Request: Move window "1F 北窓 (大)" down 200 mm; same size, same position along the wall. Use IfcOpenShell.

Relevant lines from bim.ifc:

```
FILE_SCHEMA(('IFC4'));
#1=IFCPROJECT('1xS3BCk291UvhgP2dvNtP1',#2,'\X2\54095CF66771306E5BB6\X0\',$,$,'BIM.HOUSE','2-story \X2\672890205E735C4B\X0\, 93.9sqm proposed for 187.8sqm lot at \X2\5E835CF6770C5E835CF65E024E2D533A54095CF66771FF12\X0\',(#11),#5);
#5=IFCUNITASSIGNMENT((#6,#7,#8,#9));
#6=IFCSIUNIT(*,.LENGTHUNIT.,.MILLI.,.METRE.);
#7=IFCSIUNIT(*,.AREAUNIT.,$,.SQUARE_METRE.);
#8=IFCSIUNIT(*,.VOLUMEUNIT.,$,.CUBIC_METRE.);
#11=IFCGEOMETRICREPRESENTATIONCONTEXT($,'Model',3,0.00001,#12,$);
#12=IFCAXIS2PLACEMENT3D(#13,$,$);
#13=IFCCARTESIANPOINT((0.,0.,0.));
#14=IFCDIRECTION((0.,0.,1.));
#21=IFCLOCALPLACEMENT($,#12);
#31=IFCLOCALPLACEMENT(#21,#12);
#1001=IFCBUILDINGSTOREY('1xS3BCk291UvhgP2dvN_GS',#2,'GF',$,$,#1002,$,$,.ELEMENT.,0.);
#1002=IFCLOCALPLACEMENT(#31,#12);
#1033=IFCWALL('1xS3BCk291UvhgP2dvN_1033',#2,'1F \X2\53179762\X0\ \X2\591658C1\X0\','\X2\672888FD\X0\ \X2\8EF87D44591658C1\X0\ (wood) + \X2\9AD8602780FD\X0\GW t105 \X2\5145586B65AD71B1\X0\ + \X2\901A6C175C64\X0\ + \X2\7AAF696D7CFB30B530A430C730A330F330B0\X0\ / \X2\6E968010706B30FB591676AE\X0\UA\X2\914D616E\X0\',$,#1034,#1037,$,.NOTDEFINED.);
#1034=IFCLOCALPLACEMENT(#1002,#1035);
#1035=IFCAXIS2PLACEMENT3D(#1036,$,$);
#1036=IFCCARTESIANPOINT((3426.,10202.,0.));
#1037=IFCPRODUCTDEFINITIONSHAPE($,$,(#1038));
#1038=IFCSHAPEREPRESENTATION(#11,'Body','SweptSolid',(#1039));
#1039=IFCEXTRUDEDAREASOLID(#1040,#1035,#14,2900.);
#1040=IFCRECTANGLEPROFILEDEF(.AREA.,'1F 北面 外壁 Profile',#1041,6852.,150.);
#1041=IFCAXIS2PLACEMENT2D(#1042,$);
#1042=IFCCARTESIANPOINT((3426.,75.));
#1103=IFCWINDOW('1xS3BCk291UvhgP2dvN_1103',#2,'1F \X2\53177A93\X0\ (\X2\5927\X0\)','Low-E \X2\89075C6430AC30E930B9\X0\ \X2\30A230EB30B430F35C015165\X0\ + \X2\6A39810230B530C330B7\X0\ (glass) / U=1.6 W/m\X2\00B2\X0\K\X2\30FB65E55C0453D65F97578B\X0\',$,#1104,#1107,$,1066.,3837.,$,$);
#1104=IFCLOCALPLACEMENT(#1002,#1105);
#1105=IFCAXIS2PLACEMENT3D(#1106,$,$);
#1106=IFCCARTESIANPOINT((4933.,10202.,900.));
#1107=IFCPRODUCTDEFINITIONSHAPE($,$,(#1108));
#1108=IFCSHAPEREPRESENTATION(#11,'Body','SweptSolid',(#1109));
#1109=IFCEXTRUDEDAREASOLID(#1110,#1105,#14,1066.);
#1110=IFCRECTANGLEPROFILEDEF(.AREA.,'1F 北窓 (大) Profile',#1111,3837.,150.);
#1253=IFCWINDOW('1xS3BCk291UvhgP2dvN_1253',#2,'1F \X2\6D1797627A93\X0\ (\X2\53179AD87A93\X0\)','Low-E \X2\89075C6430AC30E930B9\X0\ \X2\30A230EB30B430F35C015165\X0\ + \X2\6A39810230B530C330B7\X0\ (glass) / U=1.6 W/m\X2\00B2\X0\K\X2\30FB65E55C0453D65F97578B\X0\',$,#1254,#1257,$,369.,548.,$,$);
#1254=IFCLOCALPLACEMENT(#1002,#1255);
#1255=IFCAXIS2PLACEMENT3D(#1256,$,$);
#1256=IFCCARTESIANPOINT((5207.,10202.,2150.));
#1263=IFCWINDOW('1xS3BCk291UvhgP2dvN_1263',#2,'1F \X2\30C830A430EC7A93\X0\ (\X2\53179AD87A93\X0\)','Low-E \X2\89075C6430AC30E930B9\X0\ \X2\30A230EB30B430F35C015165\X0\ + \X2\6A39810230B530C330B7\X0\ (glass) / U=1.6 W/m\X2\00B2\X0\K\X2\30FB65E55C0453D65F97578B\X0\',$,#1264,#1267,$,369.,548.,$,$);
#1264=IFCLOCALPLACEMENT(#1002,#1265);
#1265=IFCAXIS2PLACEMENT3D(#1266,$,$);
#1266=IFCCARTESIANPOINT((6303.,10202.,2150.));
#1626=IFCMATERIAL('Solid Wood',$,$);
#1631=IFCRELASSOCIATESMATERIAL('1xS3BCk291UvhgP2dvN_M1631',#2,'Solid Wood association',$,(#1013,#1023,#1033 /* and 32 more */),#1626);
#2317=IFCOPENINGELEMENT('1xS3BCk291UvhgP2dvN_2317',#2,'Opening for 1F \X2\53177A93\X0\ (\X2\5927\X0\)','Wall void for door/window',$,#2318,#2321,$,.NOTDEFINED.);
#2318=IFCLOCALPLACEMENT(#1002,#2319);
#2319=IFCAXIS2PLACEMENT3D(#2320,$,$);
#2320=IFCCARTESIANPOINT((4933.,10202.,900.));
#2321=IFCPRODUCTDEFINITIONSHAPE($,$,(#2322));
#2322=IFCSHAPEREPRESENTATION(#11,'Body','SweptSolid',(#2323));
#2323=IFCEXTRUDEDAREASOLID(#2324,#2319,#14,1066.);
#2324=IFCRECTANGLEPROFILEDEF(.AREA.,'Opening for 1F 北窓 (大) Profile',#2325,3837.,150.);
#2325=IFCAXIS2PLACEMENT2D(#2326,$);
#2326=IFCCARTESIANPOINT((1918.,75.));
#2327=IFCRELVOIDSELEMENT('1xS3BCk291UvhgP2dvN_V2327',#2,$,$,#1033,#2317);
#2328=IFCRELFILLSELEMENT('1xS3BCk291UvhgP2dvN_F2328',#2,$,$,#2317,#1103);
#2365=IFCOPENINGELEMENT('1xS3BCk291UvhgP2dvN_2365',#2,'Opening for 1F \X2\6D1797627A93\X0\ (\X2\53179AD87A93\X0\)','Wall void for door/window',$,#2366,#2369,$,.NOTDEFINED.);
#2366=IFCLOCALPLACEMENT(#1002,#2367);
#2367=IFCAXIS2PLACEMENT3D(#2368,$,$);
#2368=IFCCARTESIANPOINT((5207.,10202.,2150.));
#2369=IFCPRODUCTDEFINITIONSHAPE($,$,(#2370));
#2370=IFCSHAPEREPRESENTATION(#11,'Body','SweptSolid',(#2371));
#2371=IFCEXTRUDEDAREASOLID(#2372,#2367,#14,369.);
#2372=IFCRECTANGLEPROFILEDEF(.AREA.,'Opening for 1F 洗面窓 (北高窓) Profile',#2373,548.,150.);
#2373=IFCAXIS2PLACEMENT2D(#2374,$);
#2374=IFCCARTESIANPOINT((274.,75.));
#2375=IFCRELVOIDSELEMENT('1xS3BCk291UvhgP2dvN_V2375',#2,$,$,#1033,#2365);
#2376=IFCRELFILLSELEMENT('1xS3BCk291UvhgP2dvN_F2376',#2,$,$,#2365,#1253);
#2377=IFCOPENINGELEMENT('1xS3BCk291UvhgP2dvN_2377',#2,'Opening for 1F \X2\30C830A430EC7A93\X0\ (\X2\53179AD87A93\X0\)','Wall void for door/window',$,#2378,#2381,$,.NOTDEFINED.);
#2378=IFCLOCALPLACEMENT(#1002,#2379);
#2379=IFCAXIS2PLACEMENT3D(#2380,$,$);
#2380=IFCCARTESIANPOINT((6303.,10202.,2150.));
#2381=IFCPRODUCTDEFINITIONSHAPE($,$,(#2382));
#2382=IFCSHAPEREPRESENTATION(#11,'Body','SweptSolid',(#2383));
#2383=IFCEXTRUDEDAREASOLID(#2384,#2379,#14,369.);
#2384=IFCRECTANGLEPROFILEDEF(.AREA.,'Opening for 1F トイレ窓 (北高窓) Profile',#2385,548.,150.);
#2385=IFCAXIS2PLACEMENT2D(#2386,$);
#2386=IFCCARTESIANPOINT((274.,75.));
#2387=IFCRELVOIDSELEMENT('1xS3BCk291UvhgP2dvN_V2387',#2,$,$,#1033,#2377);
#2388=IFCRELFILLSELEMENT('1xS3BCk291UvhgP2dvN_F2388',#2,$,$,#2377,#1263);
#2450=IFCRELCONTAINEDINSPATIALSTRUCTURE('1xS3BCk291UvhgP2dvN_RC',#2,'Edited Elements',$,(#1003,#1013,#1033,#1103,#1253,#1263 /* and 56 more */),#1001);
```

```python
import numpy as np
import ifcopenshell
import ifcopenshell.api.geometry
import ifcopenshell.util.placement
import ifcopenshell.util.unit

model = ifcopenshell.open("bim.ifc")
unit_scale = ifcopenshell.util.unit.calculate_unit_scale(model)

window = model.by_guid("1xS3BCk291UvhgP2dvN_1103")
opening = window.FillsVoids[0].RelatingOpeningElement
dz = -0.2 / unit_scale

shift = np.array([0.0, 0.0, dz])
# The window is not placed relative to its opening, so move both.
for product in (opening, window):
    matrix = ifcopenshell.util.placement.get_local_placement(product.ObjectPlacement)
    matrix[:3, 3] += shift
    ifcopenshell.api.geometry.edit_object_placement(model, product=product, matrix=matrix, is_si=False)

print(f"moved by {dz * unit_scale:+.3f} m")

model.write("bim_updated.ifc")
```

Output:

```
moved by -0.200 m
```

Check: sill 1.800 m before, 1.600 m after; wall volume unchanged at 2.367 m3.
